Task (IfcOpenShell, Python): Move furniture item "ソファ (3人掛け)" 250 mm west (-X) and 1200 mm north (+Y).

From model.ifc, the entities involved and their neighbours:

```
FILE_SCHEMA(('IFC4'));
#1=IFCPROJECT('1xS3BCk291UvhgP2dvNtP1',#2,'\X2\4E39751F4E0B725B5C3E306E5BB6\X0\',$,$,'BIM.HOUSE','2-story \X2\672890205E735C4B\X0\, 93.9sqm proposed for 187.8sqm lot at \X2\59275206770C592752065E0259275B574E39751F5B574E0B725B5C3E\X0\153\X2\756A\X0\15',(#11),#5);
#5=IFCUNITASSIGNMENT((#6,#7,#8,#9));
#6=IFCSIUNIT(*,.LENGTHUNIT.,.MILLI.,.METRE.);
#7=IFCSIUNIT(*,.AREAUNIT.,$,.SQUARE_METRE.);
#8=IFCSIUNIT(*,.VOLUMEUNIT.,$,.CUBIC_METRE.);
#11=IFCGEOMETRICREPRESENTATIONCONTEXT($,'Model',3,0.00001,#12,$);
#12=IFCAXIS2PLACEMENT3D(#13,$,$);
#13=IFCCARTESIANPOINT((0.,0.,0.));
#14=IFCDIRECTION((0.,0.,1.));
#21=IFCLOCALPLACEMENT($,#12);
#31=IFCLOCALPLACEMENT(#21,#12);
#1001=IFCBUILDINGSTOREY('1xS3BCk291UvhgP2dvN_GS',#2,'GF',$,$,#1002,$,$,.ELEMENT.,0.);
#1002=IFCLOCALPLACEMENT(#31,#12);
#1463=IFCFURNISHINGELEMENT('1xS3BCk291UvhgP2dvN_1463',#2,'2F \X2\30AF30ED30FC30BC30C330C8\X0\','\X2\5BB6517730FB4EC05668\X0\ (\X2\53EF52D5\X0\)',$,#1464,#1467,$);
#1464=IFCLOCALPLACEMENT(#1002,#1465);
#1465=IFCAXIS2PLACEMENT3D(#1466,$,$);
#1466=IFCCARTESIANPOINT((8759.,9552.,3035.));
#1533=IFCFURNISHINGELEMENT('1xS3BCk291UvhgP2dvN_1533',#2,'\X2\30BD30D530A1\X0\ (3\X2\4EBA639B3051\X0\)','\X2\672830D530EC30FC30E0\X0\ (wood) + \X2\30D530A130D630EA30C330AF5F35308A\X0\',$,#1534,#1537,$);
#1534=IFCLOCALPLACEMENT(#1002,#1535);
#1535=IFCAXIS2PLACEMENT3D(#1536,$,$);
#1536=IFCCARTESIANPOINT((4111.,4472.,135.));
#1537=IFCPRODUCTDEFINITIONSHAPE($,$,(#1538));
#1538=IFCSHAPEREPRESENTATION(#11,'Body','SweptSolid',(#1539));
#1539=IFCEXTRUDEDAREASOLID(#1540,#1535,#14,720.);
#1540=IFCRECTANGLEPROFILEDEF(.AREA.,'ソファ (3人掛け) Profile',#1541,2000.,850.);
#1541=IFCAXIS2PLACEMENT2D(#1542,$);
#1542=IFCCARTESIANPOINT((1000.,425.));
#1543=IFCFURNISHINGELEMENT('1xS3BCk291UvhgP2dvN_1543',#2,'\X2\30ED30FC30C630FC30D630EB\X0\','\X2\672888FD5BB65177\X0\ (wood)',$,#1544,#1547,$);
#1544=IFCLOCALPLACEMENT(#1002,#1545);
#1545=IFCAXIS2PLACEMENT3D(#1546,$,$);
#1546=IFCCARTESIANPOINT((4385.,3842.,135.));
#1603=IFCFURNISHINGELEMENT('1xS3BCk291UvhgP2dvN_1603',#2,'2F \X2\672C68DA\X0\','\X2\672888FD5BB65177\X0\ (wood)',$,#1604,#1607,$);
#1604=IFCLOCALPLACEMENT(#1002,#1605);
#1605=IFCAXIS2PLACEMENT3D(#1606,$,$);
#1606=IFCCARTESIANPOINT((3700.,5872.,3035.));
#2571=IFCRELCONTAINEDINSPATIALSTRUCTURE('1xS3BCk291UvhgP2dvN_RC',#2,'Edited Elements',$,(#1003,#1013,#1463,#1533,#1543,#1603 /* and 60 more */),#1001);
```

```python
import ifcopenshell
import ifcopenshell.api.geometry
import ifcopenshell.util.placement
import ifcopenshell.util.unit

model = ifcopenshell.open("model.ifc")
unit_scale = ifcopenshell.util.unit.calculate_unit_scale(model)

item = model.by_guid("1xS3BCk291UvhgP2dvN_1533")
matrix = ifcopenshell.util.placement.get_local_placement(item.ObjectPlacement)
matrix[0, 3] -= 0.25 / unit_scale
matrix[1, 3] += 1.2 / unit_scale
ifcopenshell.api.geometry.edit_object_placement(model, product=item, matrix=matrix, is_si=False)

print(ifcopenshell.util.placement.get_local_placement(item.ObjectPlacement).round(3) + 0.0)

model.write("model_v2.ifc")
```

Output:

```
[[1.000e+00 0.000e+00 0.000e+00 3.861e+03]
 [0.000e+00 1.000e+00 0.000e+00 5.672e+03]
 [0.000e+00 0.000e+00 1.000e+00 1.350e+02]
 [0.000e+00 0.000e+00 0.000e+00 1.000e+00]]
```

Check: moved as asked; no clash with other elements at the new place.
